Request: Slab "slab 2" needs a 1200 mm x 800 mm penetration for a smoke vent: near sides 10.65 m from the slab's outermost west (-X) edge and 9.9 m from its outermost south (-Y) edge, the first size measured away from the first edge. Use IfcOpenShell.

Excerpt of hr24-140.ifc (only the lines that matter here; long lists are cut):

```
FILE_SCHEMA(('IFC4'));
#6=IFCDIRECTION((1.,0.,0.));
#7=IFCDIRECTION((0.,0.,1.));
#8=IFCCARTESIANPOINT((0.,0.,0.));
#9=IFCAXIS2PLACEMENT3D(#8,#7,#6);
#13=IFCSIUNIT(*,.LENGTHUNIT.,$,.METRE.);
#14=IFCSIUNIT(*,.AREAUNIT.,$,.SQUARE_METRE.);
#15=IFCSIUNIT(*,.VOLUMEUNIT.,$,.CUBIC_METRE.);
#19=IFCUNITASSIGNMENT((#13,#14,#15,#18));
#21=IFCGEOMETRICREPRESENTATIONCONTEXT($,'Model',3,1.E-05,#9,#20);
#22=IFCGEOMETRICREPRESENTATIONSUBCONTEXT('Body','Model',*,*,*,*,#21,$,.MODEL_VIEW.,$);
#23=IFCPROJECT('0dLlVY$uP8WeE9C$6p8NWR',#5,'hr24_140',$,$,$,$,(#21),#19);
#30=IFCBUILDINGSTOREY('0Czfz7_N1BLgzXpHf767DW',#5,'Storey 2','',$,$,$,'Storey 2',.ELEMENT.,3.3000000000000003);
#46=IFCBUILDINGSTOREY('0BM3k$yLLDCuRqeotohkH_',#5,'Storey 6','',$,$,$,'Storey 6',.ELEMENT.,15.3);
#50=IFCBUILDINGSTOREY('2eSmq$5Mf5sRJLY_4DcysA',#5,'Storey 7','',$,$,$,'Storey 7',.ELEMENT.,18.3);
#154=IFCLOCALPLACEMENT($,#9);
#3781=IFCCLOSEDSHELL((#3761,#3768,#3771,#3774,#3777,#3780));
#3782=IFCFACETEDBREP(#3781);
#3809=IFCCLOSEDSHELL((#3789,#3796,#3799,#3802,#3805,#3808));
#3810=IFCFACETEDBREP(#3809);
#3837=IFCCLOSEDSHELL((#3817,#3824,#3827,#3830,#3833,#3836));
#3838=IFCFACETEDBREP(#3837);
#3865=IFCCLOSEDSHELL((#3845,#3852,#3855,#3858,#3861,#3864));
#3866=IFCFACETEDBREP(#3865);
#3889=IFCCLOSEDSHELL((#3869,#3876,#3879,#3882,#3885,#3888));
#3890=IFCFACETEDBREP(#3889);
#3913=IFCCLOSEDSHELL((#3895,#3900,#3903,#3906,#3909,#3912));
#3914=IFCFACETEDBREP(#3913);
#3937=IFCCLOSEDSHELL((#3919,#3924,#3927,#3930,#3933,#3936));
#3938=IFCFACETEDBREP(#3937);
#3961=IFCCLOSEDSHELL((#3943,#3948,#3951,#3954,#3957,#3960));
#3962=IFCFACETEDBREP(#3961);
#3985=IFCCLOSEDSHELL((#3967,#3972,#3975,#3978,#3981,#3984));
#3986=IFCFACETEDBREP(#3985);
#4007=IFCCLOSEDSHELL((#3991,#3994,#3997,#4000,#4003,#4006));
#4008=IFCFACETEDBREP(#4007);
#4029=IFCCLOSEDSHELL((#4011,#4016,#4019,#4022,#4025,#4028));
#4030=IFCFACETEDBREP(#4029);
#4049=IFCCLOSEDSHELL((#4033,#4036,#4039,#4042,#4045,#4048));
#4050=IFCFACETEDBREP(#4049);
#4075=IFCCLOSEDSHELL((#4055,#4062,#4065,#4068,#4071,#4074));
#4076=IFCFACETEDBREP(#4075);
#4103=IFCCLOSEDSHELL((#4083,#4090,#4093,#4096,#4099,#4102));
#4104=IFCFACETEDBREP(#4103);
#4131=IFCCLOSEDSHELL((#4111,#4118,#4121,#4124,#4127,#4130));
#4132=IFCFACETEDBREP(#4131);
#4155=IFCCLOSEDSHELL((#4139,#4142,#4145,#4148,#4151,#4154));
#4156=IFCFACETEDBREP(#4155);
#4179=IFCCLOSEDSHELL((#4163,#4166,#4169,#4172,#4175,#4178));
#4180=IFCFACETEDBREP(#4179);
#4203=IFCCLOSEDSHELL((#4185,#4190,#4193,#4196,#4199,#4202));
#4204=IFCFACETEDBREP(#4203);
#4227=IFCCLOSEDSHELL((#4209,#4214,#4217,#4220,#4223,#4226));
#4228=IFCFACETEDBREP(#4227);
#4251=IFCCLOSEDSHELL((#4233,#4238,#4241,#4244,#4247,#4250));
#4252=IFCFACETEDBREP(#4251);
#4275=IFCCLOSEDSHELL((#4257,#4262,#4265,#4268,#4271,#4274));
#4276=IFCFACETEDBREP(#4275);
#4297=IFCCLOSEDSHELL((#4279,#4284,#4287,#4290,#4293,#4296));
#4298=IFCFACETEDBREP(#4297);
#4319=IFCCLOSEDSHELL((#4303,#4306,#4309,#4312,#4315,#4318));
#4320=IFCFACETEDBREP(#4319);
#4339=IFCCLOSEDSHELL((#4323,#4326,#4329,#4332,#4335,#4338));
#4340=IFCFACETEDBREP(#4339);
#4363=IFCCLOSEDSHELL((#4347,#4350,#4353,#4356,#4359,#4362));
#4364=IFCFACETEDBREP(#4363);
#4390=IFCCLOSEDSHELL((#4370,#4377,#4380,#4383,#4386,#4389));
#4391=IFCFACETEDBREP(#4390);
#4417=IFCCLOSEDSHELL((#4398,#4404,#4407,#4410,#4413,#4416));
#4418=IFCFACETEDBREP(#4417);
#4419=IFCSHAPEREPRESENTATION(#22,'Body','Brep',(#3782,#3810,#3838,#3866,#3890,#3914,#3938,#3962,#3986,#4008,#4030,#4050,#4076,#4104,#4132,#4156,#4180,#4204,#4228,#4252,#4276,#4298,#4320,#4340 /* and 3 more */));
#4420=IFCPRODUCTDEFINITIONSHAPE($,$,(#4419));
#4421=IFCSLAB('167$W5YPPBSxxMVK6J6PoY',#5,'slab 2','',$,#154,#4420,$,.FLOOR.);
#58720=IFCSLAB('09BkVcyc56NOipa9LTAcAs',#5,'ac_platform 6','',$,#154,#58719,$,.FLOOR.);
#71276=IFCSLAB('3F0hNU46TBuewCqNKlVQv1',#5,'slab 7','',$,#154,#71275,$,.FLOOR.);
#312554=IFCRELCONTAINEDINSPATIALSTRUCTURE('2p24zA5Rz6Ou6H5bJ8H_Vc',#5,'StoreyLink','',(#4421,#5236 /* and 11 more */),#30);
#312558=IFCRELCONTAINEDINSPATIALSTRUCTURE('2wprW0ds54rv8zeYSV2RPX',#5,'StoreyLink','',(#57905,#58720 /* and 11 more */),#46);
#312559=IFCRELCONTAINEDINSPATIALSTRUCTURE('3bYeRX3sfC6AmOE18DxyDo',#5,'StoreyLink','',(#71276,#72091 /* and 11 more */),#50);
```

```python
import numpy as np
import ifcopenshell
import ifcopenshell.api.feature
import ifcopenshell.api.geometry
import ifcopenshell.api.root
import ifcopenshell.geom
import ifcopenshell.util.placement
import ifcopenshell.util.representation
import ifcopenshell.util.shape
import ifcopenshell.util.unit

model = ifcopenshell.open("hr24-140.ifc")
unit_scale = ifcopenshell.util.unit.calculate_unit_scale(model)
settings = ifcopenshell.geom.settings()


def volume(element):
    """Net volume in cubic metres, openings subtracted."""
    shape = ifcopenshell.geom.create_shape(settings, element)
    return ifcopenshell.util.shape.get_volume(shape.geometry)


slab = model.by_guid("167$W5YPPBSxxMVK6J6PoY")
before = volume(slab)

# Extent in the slab's own axes, in metres. The edges named are its -X and -Y sides.
slab_shape = ifcopenshell.geom.create_shape(settings, slab)
vertices = ifcopenshell.util.shape.get_vertices(slab_shape.geometry)
x_min, y_min, bottom = vertices.min(axis=0)
top = vertices[:, 2].max()

opening = ifcopenshell.api.root.create_entity(model, ifc_class="IfcOpeningElement", name="Smoke vent opening", predefined_type="OPENING")
context = ifcopenshell.util.representation.get_context(model, "Model", "Body", "MODEL_VIEW")
width, depth = 1.2, 0.8
outline = [(0.0, 0.0), (width, 0.0), (width, depth), (0.0, depth), (0.0, 0.0)]
# Overshoot both faces by 50 mm so the cut is clean.
shape = ifcopenshell.api.geometry.add_slab_representation(
    model, context=context, depth=top - bottom + 0.1, polyline=outline
)
ifcopenshell.api.geometry.assign_representation(model, product=opening, representation=shape)

matrix = ifcopenshell.util.placement.get_local_placement(slab.ObjectPlacement)
matrix[:, 3] = matrix @ np.append(np.array([x_min + 10.65, y_min + 9.9, bottom - 0.05]) / unit_scale, 1.0)
ifcopenshell.api.geometry.edit_object_placement(model, product=opening, matrix=matrix, is_si=False)
ifcopenshell.api.feature.add_feature(model, feature=opening, element=slab)

after = volume(slab)

print(f"slab volume {before:.3f} -> {after:.3f} m3")

model.write("hr24-140_updated.ifc")
```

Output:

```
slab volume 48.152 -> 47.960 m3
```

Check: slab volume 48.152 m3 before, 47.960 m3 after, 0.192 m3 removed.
